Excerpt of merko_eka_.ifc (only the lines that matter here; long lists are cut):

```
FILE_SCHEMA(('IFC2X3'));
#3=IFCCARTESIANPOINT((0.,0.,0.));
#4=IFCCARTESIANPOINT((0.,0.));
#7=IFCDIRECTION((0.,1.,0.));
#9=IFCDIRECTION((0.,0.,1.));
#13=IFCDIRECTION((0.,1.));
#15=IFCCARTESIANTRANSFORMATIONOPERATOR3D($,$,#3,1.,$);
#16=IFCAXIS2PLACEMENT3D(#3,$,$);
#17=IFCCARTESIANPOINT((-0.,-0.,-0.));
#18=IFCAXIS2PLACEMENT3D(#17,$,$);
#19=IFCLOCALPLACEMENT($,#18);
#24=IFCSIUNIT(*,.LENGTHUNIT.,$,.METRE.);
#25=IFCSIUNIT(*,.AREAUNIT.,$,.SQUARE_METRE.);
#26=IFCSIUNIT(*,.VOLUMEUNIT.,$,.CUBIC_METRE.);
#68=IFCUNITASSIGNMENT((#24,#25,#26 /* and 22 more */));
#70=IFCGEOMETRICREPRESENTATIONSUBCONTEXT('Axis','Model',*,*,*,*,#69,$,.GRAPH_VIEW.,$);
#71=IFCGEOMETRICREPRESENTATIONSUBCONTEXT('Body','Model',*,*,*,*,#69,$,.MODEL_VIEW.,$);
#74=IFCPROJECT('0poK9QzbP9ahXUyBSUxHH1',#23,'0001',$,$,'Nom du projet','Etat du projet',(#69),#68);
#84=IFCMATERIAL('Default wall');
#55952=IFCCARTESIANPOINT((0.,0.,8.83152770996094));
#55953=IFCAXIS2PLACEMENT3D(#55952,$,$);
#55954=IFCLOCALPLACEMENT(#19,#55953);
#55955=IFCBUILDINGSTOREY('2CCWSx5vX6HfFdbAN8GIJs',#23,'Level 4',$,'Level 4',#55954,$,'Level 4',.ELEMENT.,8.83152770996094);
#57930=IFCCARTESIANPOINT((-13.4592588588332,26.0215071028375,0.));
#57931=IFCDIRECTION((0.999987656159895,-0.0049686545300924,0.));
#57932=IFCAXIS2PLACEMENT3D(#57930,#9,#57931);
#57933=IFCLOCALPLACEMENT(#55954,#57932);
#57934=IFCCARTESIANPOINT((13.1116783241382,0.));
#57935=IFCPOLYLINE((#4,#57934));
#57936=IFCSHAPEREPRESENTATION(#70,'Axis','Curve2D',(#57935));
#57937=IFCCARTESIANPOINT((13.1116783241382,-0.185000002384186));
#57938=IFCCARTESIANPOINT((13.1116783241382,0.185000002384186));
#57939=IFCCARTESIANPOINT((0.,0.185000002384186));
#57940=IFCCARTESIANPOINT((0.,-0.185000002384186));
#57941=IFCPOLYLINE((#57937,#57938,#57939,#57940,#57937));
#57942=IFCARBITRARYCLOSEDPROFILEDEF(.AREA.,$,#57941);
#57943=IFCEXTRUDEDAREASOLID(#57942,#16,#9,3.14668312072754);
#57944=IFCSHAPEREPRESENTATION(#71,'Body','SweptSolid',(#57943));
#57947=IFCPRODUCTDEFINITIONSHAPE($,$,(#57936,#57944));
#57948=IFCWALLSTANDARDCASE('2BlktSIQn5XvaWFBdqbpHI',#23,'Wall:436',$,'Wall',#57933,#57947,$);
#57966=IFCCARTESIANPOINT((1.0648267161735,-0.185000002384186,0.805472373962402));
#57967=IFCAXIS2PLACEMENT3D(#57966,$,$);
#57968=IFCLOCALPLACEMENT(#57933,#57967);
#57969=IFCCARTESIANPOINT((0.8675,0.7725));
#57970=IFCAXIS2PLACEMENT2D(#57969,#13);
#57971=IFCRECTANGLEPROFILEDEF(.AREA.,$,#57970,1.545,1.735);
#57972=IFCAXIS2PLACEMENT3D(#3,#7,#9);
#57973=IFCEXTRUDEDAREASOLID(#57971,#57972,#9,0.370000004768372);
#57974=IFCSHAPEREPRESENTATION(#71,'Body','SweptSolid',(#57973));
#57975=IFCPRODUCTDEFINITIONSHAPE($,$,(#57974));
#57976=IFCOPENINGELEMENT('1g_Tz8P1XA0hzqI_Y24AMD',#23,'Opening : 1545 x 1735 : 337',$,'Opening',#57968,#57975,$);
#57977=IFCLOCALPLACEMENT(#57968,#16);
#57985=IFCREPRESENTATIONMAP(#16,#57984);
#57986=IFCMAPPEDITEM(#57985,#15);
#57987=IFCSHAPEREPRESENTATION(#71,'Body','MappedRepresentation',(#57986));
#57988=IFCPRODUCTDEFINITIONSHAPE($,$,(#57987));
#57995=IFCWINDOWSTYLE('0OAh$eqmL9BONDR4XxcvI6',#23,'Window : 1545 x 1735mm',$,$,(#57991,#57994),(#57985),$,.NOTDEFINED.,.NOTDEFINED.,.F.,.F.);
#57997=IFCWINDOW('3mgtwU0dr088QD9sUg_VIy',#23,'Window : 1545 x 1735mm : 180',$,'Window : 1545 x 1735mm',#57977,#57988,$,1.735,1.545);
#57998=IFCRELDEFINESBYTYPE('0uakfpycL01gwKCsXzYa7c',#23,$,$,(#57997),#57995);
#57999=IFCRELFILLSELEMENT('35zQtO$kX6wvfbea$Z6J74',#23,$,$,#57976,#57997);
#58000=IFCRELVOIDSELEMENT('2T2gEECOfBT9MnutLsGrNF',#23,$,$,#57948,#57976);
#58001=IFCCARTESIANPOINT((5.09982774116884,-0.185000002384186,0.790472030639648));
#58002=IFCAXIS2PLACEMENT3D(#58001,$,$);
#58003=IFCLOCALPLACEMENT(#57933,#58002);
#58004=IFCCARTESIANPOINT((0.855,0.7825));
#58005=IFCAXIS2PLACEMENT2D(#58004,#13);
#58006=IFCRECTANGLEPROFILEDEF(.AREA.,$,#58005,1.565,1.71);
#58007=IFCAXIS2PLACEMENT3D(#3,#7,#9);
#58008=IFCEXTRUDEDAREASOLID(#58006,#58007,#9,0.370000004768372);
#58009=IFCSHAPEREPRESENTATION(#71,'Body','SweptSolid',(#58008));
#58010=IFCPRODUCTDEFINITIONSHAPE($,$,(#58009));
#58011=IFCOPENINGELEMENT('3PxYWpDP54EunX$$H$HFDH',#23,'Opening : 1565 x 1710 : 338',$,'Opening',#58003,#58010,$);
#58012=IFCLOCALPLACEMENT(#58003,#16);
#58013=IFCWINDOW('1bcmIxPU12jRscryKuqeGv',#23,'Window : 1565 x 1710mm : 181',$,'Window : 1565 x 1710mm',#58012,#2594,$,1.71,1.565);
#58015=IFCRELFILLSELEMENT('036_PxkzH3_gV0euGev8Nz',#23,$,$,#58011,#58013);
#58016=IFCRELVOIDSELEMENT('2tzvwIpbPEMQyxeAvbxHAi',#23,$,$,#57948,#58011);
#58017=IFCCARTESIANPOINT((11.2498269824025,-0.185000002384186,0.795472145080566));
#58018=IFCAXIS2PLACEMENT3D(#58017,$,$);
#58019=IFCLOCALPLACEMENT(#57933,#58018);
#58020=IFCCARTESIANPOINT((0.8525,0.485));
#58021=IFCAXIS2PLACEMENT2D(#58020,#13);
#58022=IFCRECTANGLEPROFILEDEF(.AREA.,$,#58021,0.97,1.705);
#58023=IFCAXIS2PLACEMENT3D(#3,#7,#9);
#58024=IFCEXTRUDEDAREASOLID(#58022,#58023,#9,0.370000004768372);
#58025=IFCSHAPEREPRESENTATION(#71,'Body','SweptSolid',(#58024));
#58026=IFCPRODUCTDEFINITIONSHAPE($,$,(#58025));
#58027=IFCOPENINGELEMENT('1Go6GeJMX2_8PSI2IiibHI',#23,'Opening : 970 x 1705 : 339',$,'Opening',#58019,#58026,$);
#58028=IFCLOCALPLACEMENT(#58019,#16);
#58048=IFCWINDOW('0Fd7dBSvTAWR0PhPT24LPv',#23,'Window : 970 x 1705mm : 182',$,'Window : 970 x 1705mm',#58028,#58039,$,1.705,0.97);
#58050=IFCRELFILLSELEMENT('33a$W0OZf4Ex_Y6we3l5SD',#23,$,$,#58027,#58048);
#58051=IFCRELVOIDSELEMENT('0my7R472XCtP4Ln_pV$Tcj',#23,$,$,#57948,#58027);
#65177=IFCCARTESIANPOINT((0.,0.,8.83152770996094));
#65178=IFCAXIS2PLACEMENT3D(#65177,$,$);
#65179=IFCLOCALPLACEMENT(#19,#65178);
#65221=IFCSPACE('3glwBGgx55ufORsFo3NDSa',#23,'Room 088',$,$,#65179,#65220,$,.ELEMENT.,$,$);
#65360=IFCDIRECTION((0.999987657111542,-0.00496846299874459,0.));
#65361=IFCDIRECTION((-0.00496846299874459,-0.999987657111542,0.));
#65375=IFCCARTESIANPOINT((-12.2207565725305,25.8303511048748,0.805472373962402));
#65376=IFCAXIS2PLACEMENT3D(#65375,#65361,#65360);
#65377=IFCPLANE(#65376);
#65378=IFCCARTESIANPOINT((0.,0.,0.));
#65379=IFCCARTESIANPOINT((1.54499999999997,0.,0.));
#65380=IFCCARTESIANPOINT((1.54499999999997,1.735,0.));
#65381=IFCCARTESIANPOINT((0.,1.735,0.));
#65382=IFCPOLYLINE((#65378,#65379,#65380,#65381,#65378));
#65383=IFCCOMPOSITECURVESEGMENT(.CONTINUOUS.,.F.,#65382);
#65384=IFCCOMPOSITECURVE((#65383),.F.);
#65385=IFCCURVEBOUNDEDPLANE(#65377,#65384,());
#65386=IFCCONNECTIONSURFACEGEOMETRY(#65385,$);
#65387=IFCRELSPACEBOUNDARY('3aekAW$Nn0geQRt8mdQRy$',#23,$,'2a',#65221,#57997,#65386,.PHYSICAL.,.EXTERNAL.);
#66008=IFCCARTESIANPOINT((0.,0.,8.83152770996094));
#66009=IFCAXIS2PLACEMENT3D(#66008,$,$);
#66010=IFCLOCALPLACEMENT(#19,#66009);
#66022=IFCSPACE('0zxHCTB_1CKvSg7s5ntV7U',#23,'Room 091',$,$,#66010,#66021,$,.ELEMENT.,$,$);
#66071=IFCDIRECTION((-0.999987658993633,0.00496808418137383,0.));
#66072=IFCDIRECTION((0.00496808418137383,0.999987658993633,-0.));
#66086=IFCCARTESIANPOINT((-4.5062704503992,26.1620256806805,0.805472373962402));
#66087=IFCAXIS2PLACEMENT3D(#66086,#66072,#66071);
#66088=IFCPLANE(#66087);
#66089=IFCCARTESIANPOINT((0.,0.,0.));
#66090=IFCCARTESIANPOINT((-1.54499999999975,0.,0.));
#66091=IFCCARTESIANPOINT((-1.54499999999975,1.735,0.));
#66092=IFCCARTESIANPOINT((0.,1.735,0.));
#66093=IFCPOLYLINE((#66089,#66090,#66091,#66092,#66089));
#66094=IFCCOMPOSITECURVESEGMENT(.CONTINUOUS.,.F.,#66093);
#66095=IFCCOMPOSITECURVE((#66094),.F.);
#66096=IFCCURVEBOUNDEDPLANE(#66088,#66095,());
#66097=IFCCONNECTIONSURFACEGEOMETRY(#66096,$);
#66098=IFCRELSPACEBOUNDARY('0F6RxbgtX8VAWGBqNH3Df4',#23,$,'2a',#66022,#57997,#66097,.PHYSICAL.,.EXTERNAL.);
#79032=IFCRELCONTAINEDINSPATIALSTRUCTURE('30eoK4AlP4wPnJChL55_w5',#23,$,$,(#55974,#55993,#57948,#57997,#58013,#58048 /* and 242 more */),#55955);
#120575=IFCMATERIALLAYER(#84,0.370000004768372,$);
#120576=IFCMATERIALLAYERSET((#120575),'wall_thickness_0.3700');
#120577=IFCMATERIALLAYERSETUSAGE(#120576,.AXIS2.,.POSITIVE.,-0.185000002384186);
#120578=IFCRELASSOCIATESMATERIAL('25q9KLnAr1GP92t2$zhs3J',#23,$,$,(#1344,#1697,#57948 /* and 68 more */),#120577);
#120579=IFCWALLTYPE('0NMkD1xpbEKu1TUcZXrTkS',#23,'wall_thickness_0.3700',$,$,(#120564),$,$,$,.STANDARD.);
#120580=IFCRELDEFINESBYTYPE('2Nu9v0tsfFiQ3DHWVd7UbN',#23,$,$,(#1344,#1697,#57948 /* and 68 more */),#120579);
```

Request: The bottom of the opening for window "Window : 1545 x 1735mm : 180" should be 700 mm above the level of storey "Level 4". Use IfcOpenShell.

```python
import numpy as np
import ifcopenshell
import ifcopenshell.api.geometry
import ifcopenshell.geom
import ifcopenshell.util.element
import ifcopenshell.util.placement
import ifcopenshell.util.shape
import ifcopenshell.util.unit

model = ifcopenshell.open("merko_eka_.ifc")
unit_scale = ifcopenshell.util.unit.calculate_unit_scale(model)

window = model.by_id(57997)
opening = window.FillsVoids[0].RelatingOpeningElement
storey = ifcopenshell.util.element.get_container(window, ifc_class="IfcBuildingStorey")
level = ifcopenshell.util.placement.get_local_placement(storey.ObjectPlacement)[2, 3]

# The opening's origin need not be at the sill, so measure its lowest point.
shape = ifcopenshell.geom.create_shape(ifcopenshell.geom.settings(), opening)
bottom = ifcopenshell.util.shape.get_shape_bottom_elevation(shape, shape.geometry) / unit_scale
dz = level + 0.7 / unit_scale - bottom

shift = np.array([0.0, 0.0, dz])
# The window is placed relative to its opening, so it follows when the opening moves.
matrix = ifcopenshell.util.placement.get_local_placement(opening.ObjectPlacement)
matrix[:3, 3] += shift
ifcopenshell.api.geometry.edit_object_placement(
    model, product=opening, matrix=matrix, is_si=False, should_transform_children=True
)

# Space boundary surfaces are stored in each space's coordinates; move them too.
for rel in window.ProvidesBoundaries:
    if not rel.ConnectionGeometry:
        continue
    surface = rel.ConnectionGeometry.SurfaceOnRelatingElement.BasisSurface
    space_matrix = ifcopenshell.util.placement.get_local_placement(rel.RelatingSpace.ObjectPlacement)
    point = np.array(surface.Position.Location.Coordinates) + space_matrix[:3, :3].T @ shift
    surface.Position = model.createIfcAxis2Placement3D(
        model.createIfcCartesianPoint(point.tolist()), surface.Position.Axis, surface.Position.RefDirection
    )

print(f"moved by {dz * unit_scale:+.3f} m")

model.write("merko_eka__edited.ifc")
```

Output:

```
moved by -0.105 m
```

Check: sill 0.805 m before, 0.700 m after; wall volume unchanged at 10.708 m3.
